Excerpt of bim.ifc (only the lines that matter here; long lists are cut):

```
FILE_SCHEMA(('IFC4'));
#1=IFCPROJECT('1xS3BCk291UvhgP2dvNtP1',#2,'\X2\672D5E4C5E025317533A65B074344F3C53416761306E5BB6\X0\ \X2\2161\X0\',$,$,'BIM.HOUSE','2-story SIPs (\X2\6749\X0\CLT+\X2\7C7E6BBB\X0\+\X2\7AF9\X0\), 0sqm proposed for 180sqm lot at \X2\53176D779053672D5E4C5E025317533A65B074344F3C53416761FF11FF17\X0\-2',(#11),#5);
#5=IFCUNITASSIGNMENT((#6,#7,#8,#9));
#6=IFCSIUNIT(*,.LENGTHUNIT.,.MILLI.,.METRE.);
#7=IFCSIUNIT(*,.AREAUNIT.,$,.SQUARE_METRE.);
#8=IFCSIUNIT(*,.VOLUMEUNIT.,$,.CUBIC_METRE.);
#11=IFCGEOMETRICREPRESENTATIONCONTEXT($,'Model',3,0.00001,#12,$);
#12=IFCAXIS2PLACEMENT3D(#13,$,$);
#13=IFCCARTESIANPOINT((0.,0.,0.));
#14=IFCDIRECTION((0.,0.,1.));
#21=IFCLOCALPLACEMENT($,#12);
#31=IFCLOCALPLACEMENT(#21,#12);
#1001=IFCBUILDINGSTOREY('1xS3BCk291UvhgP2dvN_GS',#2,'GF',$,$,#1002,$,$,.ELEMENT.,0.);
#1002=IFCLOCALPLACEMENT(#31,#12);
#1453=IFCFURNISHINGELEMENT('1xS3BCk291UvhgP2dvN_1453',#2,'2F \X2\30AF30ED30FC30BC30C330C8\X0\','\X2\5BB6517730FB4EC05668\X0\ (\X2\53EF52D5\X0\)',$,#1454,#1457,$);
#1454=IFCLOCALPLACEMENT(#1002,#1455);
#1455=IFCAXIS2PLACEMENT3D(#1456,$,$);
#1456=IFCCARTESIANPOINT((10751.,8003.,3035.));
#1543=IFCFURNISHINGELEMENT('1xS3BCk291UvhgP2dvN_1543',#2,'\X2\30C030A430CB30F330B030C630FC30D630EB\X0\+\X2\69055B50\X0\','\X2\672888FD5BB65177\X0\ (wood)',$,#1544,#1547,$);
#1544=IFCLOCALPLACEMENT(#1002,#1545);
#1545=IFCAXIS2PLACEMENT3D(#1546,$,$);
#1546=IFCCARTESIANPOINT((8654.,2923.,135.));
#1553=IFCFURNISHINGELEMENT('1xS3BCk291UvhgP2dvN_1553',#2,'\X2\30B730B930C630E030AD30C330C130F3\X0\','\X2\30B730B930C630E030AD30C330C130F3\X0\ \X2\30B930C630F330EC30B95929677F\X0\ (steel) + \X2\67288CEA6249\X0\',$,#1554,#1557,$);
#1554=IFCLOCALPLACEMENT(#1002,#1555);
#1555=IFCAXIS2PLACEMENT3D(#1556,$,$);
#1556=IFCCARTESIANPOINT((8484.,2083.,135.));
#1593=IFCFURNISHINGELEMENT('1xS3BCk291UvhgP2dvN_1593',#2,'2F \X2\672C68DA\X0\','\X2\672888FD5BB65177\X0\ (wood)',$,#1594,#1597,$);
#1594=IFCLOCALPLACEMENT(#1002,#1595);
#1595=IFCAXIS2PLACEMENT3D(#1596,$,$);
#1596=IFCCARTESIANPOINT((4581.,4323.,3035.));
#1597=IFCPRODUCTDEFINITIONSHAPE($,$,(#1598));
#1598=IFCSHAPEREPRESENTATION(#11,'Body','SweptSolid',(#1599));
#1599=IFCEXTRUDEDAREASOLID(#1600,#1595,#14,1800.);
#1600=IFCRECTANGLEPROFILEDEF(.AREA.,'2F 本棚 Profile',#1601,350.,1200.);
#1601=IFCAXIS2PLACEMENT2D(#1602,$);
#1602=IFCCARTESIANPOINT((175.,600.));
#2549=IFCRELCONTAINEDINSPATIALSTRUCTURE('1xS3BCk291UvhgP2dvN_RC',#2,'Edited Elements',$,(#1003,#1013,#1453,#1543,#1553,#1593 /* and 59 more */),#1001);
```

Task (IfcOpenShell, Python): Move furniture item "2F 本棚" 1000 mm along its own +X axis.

```python
import ifcopenshell
import ifcopenshell.api.geometry
import ifcopenshell.util.placement
import ifcopenshell.util.unit

model = ifcopenshell.open("bim.ifc")
unit_scale = ifcopenshell.util.unit.calculate_unit_scale(model)

item = model.by_guid("1xS3BCk291UvhgP2dvN_1593")
matrix = ifcopenshell.util.placement.get_local_placement(item.ObjectPlacement)
matrix[:3, 3] += matrix[:3, 0] * 1 / unit_scale
ifcopenshell.api.geometry.edit_object_placement(model, product=item, matrix=matrix, is_si=False)

print(ifcopenshell.util.placement.get_local_placement(item.ObjectPlacement).round(3) + 0.0)

model.write("bim_updated.ifc")
```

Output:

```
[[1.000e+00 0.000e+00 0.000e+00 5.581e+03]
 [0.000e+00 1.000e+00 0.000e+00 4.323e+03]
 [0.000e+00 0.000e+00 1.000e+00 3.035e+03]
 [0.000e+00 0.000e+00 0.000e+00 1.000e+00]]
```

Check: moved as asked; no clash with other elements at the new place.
